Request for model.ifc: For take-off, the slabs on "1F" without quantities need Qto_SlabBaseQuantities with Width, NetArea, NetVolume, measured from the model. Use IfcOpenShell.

First a look at what the model holds.

```python
import ifcopenshell
import ifcopenshell.util.element
import ifcopenshell.util.unit

model = ifcopenshell.open("model.ifc")
print(model.schema)
for unit_type in ("LENGTHUNIT", "AREAUNIT", "VOLUMEUNIT"):
    print(unit_type, ifcopenshell.util.unit.calculate_unit_scale(model, unit_type))
storey = next(s for s in model.by_type("IfcBuildingStorey") if s.Name == "1F")
slabs = [e for e in ifcopenshell.util.element.get_decomposition(storey) if e.is_a("IfcSlab")]
for e in sorted(slabs, key=lambda e: e.id()):
    print(e.id(), e.is_a(), e.Name, list(ifcopenshell.util.element.get_psets(e, qtos_only=True)), sep=" | ")
```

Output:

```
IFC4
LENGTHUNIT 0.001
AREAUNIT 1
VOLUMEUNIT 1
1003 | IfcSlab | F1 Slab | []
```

```python
import ifcopenshell
import ifcopenshell.api.pset
import ifcopenshell.geom
import ifcopenshell.util.element
import ifcopenshell.util.shape
import ifcopenshell.util.unit

model = ifcopenshell.open("model.ifc")
unit_scale = ifcopenshell.util.unit.calculate_unit_scale(model)
area_scale = ifcopenshell.util.unit.calculate_unit_scale(model, "AREAUNIT")
volume_scale = ifcopenshell.util.unit.calculate_unit_scale(model, "VOLUMEUNIT")
settings = ifcopenshell.geom.settings()

storey = next(s for s in model.by_type("IfcBuildingStorey") if s.Name == "1F")
slabs = [e for e in ifcopenshell.util.element.get_decomposition(storey) if e.is_a("IfcSlab")]

for e in sorted(slabs, key=lambda e: e.id()):
    if ifcopenshell.util.element.get_psets(e, qtos_only=True, should_inherit=False):
        continue
    # Geometry comes back in metres, in the element's own axes.
    shape = ifcopenshell.geom.create_shape(settings, e)
    values = {
        "Width": ifcopenshell.util.shape.get_z(shape.geometry) / unit_scale,
        "NetArea": ifcopenshell.util.shape.get_footprint_area(shape.geometry) / area_scale,
        "NetVolume": ifcopenshell.util.shape.get_volume(shape.geometry) / volume_scale,
    }
    qto = ifcopenshell.api.pset.add_qto(model, product=e, name="Qto_SlabBaseQuantities")
    ifcopenshell.api.pset.edit_qto(model, qto=qto, properties=values)
    print(e.id(), {k: round(v, 3) for k, v in values.items()})

model.write("model_rev.ifc")
```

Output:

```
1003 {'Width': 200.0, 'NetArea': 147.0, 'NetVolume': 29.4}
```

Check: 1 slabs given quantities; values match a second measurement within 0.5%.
